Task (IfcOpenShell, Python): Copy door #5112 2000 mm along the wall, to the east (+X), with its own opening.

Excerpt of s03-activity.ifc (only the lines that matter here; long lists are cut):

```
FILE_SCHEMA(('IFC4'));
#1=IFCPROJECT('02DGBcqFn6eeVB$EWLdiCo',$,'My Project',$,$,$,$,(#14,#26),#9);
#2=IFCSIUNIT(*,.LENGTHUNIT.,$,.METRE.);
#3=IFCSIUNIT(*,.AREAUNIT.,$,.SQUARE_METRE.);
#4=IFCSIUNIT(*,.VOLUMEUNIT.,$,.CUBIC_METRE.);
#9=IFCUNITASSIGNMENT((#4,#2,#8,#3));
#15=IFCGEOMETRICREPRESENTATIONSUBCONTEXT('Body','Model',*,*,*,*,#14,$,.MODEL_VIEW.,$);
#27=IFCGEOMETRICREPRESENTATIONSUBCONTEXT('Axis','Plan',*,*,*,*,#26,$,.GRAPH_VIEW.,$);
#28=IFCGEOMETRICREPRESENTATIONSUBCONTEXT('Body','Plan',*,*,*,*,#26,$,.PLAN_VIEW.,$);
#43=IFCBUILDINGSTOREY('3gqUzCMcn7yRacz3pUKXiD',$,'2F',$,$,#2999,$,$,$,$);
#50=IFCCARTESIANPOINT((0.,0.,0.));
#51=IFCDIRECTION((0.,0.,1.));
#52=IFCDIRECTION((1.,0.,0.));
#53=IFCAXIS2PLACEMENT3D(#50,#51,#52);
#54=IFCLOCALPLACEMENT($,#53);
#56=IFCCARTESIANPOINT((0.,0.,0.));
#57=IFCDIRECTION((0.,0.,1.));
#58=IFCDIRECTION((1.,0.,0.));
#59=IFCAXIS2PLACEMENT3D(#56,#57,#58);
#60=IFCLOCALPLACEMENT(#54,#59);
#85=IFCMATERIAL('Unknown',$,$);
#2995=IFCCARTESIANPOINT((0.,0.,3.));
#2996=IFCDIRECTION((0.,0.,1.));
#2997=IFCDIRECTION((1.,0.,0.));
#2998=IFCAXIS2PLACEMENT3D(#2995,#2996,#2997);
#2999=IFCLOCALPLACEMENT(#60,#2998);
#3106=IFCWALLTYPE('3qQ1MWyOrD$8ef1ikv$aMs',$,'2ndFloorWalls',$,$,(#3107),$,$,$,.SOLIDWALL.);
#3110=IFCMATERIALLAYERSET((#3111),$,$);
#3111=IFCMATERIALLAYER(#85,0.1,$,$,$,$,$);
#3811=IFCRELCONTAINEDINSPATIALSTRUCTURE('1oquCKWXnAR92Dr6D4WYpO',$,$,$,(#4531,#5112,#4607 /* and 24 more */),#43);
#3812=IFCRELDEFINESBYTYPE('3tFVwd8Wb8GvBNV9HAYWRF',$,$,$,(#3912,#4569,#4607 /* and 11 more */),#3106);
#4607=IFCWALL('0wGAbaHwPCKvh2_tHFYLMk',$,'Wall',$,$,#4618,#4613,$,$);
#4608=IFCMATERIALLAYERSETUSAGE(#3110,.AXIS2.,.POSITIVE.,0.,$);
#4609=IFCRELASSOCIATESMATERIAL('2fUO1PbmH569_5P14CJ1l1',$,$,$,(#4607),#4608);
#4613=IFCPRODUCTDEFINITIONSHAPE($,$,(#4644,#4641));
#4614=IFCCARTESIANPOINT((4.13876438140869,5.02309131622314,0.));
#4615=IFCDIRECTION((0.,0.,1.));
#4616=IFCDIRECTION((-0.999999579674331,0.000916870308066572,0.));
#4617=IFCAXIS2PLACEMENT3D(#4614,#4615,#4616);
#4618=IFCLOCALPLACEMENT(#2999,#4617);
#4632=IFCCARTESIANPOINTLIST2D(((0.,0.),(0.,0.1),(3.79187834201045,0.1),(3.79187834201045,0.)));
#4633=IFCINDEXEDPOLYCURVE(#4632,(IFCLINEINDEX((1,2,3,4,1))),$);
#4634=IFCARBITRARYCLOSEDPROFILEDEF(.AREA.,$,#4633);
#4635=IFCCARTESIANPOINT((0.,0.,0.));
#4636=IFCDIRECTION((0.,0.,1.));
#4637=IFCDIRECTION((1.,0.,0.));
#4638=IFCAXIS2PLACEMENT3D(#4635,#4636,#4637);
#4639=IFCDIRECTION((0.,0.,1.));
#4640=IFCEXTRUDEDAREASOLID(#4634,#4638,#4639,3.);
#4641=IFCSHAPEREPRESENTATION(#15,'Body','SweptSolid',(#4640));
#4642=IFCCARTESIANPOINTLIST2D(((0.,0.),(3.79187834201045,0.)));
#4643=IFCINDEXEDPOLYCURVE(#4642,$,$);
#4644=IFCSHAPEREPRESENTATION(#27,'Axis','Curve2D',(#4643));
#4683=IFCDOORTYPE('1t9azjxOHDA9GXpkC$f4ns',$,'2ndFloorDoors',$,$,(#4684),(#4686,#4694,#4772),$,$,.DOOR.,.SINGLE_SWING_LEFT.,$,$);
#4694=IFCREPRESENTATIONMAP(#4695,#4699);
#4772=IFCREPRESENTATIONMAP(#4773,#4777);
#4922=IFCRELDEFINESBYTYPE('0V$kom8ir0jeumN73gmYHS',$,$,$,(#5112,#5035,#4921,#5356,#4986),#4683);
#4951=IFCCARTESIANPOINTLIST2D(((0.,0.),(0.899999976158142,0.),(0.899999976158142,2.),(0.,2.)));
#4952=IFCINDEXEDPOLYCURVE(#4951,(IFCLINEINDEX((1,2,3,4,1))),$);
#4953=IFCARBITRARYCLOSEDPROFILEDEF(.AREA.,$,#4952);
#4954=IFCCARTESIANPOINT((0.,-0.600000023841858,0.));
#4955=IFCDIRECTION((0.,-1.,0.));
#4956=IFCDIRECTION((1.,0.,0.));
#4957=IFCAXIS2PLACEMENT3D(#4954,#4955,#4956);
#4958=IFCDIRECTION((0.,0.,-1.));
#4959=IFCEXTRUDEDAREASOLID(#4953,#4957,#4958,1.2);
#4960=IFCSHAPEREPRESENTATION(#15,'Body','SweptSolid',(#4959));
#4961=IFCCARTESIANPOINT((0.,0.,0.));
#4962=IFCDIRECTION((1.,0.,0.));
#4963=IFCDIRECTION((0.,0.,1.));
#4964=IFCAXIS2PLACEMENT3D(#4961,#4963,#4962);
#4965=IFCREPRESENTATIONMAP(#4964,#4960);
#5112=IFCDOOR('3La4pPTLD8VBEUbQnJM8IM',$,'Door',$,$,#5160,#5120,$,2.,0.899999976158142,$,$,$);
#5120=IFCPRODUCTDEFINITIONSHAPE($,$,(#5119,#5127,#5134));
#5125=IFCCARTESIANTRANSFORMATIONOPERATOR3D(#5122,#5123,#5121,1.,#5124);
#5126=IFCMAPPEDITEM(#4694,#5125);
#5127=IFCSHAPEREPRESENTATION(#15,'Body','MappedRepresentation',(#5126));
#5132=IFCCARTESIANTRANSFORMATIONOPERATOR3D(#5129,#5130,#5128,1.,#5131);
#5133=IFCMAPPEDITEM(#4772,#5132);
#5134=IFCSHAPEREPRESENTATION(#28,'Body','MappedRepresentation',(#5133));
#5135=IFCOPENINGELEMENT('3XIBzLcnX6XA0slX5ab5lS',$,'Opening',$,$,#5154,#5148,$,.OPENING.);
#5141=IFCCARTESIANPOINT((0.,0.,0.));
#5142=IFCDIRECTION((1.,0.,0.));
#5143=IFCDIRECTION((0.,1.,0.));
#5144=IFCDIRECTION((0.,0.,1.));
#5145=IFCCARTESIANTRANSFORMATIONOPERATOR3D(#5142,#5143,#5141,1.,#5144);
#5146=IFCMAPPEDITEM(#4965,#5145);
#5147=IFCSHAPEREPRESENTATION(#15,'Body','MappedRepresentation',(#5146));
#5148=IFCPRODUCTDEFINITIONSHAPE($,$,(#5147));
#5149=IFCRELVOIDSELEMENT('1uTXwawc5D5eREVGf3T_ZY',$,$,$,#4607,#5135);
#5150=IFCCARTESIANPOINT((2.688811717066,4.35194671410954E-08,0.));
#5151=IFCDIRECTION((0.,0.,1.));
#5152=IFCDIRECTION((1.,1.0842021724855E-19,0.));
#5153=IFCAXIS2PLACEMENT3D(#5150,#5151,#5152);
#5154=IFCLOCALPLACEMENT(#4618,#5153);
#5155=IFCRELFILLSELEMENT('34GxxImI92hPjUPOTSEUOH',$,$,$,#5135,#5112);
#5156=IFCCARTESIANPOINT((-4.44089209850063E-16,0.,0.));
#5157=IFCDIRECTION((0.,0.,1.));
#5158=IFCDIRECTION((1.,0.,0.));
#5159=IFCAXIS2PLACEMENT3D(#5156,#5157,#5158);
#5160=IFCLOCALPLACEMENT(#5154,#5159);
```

```python
import ifcopenshell
import ifcopenshell.api.feature
import ifcopenshell.api.geometry
import ifcopenshell.api.root
import ifcopenshell.geom
import ifcopenshell.util.element
import ifcopenshell.util.placement
import ifcopenshell.util.shape

model = ifcopenshell.open("s03-activity.ifc")
settings = ifcopenshell.geom.settings()


def volume(element):
    """Net volume in cubic metres, openings subtracted."""
    shape = ifcopenshell.geom.create_shape(settings, element)
    return ifcopenshell.util.shape.get_volume(shape.geometry)


door = model.by_id(5112)
opening = door.FillsVoids[0].RelatingOpeningElement
wall = opening.VoidsElements[0].RelatingBuildingElement
before = volume(wall)
shift = ifcopenshell.util.placement.get_local_placement(wall.ObjectPlacement)[:3, 0] * -2.0

# copy_class copies the void relationship, type, container and properties, but no geometry.
new_opening = ifcopenshell.api.root.copy_class(model, product=opening)
new_opening.Representation = ifcopenshell.util.element.copy_deep(
    model, opening.Representation, exclude=["IfcGeometricRepresentationContext", "IfcRepresentationMap"]
)
new_door = ifcopenshell.api.root.copy_class(model, product=door)
new_door.Representation = ifcopenshell.util.element.copy_deep(
    model, door.Representation, exclude=["IfcGeometricRepresentationContext", "IfcRepresentationMap"]
)
ifcopenshell.api.feature.add_filling(model, opening=new_opening, element=new_door)

for old, new in ((opening, new_opening), (door, new_door)):
    matrix = ifcopenshell.util.placement.get_local_placement(old.ObjectPlacement)
    matrix[:3, 3] += shift
    ifcopenshell.api.geometry.edit_object_placement(model, product=new, matrix=matrix, is_si=False)

after = volume(wall)

print(f"wall volume {before:.3f} -> {after:.3f} m3")

model.write("s03-activity_v2.ifc")
```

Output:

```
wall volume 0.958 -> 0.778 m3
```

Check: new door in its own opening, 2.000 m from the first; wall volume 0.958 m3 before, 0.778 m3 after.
